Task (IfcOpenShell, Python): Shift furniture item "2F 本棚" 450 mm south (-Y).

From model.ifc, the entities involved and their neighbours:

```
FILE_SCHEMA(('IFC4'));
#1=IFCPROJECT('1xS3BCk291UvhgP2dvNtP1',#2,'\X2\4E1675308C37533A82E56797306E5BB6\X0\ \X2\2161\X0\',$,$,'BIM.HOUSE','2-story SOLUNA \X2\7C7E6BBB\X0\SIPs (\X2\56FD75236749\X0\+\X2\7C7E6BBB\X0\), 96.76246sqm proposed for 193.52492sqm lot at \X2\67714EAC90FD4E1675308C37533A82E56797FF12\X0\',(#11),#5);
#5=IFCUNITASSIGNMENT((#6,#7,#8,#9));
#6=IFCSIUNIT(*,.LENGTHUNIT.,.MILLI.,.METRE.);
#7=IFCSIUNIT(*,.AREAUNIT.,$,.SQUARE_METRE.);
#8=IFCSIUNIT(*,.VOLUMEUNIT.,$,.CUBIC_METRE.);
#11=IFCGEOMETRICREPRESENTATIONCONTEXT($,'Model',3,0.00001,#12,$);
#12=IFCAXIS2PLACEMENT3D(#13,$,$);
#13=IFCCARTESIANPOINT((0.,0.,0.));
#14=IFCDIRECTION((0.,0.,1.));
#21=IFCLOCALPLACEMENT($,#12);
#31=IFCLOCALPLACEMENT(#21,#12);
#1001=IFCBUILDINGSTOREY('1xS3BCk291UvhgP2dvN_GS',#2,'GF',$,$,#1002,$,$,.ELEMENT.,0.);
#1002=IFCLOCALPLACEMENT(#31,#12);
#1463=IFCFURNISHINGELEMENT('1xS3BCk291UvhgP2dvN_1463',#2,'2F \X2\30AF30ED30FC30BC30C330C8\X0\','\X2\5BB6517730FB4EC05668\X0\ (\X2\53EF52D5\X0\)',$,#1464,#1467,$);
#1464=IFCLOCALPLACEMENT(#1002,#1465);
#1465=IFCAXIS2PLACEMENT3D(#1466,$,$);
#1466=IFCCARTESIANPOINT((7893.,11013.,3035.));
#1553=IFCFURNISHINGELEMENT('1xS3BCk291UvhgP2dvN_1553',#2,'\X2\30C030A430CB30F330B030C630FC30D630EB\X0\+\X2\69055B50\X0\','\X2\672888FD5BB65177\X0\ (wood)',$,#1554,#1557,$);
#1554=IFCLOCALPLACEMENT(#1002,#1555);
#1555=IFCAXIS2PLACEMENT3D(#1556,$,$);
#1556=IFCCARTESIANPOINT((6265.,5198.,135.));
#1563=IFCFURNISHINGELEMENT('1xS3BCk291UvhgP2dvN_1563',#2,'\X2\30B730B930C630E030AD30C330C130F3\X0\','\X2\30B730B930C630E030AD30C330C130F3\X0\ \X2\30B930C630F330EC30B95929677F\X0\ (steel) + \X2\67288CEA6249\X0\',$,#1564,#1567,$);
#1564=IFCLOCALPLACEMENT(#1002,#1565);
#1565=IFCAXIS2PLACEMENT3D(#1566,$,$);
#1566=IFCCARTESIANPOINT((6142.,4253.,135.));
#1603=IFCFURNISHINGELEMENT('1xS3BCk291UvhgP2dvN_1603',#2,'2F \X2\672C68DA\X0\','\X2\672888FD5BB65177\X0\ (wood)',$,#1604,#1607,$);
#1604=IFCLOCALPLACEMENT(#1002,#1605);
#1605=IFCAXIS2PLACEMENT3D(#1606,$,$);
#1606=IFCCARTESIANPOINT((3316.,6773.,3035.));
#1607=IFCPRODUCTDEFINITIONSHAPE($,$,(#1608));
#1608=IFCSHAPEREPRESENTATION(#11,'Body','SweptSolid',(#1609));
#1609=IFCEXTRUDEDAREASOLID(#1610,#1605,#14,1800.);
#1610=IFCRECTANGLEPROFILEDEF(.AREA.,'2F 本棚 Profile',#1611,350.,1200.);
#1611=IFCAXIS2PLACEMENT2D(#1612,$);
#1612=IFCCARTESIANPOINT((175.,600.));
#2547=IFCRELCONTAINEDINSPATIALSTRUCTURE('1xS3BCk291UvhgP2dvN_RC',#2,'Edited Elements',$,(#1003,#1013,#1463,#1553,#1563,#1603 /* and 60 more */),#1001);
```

```python
import ifcopenshell
import ifcopenshell.api.geometry
import ifcopenshell.util.placement

model = ifcopenshell.open("model.ifc")

item = model.by_guid("1xS3BCk291UvhgP2dvN_1603")
matrix = ifcopenshell.util.placement.get_local_placement(item.ObjectPlacement)
matrix[1, 3] -= 450.0
ifcopenshell.api.geometry.edit_object_placement(model, product=item, matrix=matrix, is_si=False)

print(ifcopenshell.util.placement.get_local_placement(item.ObjectPlacement).round(3) + 0.0)

model.write("model-out.ifc")
```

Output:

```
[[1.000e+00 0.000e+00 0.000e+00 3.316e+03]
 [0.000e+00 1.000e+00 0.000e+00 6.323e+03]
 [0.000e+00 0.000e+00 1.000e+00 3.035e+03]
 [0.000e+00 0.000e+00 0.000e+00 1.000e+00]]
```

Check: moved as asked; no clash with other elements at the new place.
